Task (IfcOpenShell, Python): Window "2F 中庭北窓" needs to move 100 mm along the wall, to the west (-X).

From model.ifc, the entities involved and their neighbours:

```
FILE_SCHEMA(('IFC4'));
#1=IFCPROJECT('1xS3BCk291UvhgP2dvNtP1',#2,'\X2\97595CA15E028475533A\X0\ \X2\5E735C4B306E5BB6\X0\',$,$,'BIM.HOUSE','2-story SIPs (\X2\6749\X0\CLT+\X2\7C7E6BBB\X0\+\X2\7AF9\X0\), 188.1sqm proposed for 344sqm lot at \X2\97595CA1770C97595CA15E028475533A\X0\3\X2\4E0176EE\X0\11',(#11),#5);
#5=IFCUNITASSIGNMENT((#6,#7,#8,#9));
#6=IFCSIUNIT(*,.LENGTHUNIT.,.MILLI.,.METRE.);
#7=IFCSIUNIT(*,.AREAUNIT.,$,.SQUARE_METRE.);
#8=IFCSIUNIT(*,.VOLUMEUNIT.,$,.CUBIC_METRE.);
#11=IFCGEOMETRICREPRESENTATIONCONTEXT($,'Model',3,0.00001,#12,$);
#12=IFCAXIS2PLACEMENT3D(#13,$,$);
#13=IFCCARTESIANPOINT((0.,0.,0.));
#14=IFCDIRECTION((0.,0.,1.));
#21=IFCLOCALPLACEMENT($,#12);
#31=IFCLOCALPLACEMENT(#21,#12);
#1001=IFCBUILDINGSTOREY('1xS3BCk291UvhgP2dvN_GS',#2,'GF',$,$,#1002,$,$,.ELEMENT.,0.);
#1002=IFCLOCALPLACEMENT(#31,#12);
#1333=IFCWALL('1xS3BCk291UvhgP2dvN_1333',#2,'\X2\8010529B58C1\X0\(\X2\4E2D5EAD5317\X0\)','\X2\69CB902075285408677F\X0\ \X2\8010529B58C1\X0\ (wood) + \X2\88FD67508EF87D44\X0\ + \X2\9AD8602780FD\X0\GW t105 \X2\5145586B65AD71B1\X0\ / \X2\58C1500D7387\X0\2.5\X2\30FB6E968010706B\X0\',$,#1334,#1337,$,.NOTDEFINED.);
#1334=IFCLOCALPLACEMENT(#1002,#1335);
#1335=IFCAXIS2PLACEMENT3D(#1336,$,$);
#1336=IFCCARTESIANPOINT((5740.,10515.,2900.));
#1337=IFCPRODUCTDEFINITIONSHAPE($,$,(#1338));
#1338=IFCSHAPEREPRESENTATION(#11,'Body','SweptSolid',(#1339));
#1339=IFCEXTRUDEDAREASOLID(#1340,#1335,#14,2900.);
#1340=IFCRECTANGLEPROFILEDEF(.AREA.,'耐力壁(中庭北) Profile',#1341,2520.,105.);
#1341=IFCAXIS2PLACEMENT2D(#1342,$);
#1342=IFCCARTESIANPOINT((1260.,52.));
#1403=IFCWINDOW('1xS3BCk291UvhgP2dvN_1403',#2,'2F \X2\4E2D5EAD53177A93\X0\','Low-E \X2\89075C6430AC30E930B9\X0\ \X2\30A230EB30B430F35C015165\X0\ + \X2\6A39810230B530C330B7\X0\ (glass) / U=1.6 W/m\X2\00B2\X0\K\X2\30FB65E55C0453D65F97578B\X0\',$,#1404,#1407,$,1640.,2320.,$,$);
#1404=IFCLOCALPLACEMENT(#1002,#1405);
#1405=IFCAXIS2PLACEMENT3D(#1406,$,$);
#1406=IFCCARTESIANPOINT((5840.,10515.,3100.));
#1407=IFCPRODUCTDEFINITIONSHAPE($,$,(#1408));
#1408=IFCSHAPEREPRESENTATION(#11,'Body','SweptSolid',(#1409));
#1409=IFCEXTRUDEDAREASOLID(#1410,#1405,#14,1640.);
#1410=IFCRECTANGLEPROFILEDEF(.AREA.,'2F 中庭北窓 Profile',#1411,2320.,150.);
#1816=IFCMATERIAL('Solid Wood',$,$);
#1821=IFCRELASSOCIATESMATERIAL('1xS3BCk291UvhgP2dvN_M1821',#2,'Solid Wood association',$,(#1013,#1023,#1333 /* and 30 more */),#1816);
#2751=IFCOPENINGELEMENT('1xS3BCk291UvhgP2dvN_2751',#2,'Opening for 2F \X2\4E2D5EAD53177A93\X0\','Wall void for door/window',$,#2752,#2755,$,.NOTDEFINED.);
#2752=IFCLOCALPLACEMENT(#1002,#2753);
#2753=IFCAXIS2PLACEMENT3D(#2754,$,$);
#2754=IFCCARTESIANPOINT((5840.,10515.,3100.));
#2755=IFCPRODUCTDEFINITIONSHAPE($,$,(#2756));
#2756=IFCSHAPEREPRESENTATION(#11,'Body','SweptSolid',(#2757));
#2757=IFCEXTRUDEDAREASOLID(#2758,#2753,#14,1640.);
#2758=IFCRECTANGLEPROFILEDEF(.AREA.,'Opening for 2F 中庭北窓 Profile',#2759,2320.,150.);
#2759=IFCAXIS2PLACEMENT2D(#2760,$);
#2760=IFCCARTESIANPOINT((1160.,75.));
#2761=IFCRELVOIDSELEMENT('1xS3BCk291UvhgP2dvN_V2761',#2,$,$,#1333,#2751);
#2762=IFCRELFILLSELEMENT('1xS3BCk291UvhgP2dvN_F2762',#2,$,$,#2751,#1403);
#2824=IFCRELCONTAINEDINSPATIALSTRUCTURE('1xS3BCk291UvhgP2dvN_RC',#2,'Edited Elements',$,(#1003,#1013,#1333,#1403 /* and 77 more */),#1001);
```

```python
import ifcopenshell
import ifcopenshell.api.geometry
import ifcopenshell.util.placement

model = ifcopenshell.open("model.ifc")

window = model.by_guid("1xS3BCk291UvhgP2dvN_1403")
opening = window.FillsVoids[0].RelatingOpeningElement
wall = opening.VoidsElements[0].RelatingBuildingElement

wall_matrix = ifcopenshell.util.placement.get_local_placement(wall.ObjectPlacement)
shift = wall_matrix[:3, 0] * -100.0
before = ifcopenshell.util.placement.get_local_placement(window.ObjectPlacement)[:3, 3].copy()

# The window is not placed relative to its opening, so move both.
for product in (opening, window):
    matrix = ifcopenshell.util.placement.get_local_placement(product.ObjectPlacement)
    matrix[:3, 3] += shift
    ifcopenshell.api.geometry.edit_object_placement(model, product=product, matrix=matrix, is_si=False)

after = ifcopenshell.util.placement.get_local_placement(window.ObjectPlacement)[:3, 3]
print("window moved by", (after - before).round(3) + 0.0)

model.write("model_v2.ifc")
```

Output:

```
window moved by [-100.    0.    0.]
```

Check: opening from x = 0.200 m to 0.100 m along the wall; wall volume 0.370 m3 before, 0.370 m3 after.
